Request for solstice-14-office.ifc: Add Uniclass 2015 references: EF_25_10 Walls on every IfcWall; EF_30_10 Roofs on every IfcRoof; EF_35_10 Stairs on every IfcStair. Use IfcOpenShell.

First a look at what the model holds.

```python
import ifcopenshell

model = ifcopenshell.open("solstice-14-office.ifc")
print(model.schema)
print("classifications:", [c.Name for c in model.by_type("IfcClassification")])
for ifc_class in ("IfcDoor", "IfcRoof", "IfcStair", "IfcWall", "IfcWindow"):
    print(ifc_class, len(model.by_type(ifc_class)))
```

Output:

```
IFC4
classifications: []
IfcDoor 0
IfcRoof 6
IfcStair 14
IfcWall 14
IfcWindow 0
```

```python
import ifcopenshell
import ifcopenshell.api.classification

model = ifcopenshell.open("solstice-14-office.ifc")

system = ifcopenshell.api.classification.add_classification(model, classification="Uniclass 2015")

codes = {
    "IfcWall": ("EF_25_10", "Walls"),
    "IfcRoof": ("EF_30_10", "Roofs"),
    "IfcStair": ("EF_35_10", "Stairs"),
}
for ifc_class, (code, name) in codes.items():
    products = model.by_type(ifc_class)
    ifcopenshell.api.classification.add_reference(
        model, products=products, classification=system, identification=code, name=name
    )
    print(code, len(products))

model.write("solstice-14-office_v2.ifc")
```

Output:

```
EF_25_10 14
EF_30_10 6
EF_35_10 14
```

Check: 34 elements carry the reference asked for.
